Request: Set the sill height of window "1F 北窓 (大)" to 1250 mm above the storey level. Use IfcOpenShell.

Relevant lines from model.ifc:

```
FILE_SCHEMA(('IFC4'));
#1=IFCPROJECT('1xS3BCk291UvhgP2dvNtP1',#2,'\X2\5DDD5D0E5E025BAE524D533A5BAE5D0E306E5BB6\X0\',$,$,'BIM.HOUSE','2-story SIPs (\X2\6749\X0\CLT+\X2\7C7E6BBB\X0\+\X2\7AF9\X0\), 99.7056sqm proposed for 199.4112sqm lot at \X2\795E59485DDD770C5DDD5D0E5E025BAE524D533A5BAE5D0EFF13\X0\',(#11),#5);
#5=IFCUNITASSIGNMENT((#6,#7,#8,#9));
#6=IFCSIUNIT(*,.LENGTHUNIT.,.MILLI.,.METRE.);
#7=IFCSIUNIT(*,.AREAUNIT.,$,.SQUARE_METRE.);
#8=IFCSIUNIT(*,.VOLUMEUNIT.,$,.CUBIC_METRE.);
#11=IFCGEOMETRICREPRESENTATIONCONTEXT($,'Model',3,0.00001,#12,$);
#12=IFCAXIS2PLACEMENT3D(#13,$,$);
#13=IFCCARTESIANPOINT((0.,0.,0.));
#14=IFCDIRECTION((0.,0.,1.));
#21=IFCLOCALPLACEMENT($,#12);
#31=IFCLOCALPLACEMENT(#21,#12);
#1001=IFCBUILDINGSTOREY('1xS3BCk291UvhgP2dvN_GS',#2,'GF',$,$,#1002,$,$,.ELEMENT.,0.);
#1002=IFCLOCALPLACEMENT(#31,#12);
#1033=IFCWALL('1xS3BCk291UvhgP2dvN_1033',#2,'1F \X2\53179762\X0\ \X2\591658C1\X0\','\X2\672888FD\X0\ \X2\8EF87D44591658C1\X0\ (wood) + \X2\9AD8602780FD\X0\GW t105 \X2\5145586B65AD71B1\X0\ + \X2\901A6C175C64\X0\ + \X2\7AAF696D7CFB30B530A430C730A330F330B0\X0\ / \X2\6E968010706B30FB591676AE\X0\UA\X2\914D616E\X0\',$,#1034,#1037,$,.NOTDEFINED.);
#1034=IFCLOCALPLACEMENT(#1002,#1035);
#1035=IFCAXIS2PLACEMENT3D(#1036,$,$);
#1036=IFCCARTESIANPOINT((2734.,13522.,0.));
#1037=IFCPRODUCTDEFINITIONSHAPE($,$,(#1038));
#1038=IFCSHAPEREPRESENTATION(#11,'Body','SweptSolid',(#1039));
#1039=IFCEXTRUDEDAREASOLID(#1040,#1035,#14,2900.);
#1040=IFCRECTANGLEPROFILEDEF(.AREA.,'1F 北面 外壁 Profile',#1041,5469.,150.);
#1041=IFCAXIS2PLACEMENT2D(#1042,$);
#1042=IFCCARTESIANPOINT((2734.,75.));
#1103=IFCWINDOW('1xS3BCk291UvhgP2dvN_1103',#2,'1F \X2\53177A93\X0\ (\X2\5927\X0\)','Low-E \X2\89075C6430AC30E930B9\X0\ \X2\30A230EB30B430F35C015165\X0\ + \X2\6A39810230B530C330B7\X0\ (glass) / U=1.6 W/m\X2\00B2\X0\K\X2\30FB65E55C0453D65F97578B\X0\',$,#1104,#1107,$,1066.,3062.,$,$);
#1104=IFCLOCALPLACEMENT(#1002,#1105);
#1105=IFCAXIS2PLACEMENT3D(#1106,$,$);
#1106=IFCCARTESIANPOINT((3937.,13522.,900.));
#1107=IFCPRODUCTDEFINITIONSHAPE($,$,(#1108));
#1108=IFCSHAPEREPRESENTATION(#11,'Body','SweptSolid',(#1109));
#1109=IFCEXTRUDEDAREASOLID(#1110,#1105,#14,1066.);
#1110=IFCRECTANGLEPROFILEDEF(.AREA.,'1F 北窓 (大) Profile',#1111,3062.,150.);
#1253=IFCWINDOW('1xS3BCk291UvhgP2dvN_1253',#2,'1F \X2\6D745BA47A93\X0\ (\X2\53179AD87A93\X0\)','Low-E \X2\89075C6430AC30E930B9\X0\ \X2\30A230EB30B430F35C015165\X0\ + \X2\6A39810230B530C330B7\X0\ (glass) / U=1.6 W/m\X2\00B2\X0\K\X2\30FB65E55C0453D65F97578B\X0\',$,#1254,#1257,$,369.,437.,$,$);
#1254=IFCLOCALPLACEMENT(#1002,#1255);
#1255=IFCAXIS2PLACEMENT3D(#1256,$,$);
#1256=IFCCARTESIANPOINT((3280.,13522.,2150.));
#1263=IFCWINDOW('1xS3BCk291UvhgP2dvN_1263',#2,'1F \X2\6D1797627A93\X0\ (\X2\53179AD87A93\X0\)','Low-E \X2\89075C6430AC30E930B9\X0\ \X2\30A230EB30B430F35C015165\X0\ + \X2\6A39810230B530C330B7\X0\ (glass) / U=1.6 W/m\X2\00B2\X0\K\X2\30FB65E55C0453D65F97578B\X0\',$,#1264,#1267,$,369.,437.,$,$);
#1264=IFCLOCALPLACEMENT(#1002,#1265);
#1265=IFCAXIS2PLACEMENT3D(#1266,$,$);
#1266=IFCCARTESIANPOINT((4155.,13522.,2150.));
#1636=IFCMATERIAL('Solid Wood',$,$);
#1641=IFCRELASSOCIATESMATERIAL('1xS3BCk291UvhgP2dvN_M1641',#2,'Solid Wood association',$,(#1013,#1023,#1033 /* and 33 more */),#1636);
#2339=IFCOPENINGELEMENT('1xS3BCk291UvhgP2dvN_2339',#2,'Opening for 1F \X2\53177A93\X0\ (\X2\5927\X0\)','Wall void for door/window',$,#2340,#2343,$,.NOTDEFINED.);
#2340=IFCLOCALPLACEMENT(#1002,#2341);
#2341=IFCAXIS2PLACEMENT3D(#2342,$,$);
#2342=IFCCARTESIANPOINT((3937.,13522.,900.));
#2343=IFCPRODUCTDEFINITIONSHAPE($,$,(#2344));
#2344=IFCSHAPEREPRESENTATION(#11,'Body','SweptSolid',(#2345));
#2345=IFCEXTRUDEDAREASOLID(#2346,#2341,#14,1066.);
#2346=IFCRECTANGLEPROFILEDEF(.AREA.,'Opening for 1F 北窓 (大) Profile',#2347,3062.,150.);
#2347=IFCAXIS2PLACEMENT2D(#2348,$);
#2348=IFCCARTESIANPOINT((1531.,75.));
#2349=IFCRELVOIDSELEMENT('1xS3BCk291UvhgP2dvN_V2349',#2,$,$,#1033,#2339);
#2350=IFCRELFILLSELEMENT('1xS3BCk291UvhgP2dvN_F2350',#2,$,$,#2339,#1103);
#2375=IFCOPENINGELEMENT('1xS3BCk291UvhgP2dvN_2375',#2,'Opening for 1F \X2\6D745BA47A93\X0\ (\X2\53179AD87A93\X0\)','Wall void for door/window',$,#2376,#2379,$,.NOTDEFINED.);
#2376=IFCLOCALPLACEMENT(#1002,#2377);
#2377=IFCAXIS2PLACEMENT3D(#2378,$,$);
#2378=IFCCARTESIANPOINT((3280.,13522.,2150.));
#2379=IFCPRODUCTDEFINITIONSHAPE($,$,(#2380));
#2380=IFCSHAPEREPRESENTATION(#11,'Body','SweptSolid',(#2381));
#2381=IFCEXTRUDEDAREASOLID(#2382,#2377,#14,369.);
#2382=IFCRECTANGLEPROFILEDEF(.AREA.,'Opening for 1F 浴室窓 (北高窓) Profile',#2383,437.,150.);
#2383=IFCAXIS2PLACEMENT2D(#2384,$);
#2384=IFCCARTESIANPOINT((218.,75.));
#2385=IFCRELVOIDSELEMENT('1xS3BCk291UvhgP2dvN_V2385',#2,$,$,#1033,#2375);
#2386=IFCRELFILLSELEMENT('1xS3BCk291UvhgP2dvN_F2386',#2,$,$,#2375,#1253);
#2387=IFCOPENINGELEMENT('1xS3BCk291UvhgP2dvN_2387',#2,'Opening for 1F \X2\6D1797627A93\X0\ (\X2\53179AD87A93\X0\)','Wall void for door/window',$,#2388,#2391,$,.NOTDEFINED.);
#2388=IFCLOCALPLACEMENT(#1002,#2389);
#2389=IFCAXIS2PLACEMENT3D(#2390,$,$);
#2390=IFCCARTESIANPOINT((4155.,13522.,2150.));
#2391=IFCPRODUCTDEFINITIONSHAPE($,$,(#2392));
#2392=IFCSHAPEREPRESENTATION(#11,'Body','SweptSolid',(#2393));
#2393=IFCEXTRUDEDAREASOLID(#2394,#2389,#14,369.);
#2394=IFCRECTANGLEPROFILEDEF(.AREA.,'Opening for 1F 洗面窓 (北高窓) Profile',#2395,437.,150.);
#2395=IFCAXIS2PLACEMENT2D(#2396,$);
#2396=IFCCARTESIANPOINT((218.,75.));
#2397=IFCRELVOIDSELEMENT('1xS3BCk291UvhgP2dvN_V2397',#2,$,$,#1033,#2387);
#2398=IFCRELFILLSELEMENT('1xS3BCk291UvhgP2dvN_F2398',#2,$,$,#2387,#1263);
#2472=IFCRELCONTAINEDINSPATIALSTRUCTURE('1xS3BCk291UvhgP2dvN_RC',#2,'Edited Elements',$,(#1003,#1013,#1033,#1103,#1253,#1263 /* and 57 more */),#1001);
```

```python
import numpy as np
import ifcopenshell
import ifcopenshell.api.geometry
import ifcopenshell.geom
import ifcopenshell.util.element
import ifcopenshell.util.placement
import ifcopenshell.util.shape
import ifcopenshell.util.unit

model = ifcopenshell.open("model.ifc")
unit_scale = ifcopenshell.util.unit.calculate_unit_scale(model)

window = model.by_id(1103)
opening = window.FillsVoids[0].RelatingOpeningElement
storey = ifcopenshell.util.element.get_container(window, ifc_class="IfcBuildingStorey")
level = ifcopenshell.util.placement.get_local_placement(storey.ObjectPlacement)[2, 3]

# The opening's origin need not be at the sill, so measure its lowest point.
shape = ifcopenshell.geom.create_shape(ifcopenshell.geom.settings(), opening)
bottom = ifcopenshell.util.shape.get_shape_bottom_elevation(shape, shape.geometry) / unit_scale
dz = level + 1.25 / unit_scale - bottom

shift = np.array([0.0, 0.0, dz])
# The window is not placed relative to its opening, so move both.
for product in (opening, window):
    matrix = ifcopenshell.util.placement.get_local_placement(product.ObjectPlacement)
    matrix[:3, 3] += shift
    ifcopenshell.api.geometry.edit_object_placement(model, product=product, matrix=matrix, is_si=False)

print(f"moved by {dz * unit_scale:+.3f} m")

model.write("model_rev.ifc")
```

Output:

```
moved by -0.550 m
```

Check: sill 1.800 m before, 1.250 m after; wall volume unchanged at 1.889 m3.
